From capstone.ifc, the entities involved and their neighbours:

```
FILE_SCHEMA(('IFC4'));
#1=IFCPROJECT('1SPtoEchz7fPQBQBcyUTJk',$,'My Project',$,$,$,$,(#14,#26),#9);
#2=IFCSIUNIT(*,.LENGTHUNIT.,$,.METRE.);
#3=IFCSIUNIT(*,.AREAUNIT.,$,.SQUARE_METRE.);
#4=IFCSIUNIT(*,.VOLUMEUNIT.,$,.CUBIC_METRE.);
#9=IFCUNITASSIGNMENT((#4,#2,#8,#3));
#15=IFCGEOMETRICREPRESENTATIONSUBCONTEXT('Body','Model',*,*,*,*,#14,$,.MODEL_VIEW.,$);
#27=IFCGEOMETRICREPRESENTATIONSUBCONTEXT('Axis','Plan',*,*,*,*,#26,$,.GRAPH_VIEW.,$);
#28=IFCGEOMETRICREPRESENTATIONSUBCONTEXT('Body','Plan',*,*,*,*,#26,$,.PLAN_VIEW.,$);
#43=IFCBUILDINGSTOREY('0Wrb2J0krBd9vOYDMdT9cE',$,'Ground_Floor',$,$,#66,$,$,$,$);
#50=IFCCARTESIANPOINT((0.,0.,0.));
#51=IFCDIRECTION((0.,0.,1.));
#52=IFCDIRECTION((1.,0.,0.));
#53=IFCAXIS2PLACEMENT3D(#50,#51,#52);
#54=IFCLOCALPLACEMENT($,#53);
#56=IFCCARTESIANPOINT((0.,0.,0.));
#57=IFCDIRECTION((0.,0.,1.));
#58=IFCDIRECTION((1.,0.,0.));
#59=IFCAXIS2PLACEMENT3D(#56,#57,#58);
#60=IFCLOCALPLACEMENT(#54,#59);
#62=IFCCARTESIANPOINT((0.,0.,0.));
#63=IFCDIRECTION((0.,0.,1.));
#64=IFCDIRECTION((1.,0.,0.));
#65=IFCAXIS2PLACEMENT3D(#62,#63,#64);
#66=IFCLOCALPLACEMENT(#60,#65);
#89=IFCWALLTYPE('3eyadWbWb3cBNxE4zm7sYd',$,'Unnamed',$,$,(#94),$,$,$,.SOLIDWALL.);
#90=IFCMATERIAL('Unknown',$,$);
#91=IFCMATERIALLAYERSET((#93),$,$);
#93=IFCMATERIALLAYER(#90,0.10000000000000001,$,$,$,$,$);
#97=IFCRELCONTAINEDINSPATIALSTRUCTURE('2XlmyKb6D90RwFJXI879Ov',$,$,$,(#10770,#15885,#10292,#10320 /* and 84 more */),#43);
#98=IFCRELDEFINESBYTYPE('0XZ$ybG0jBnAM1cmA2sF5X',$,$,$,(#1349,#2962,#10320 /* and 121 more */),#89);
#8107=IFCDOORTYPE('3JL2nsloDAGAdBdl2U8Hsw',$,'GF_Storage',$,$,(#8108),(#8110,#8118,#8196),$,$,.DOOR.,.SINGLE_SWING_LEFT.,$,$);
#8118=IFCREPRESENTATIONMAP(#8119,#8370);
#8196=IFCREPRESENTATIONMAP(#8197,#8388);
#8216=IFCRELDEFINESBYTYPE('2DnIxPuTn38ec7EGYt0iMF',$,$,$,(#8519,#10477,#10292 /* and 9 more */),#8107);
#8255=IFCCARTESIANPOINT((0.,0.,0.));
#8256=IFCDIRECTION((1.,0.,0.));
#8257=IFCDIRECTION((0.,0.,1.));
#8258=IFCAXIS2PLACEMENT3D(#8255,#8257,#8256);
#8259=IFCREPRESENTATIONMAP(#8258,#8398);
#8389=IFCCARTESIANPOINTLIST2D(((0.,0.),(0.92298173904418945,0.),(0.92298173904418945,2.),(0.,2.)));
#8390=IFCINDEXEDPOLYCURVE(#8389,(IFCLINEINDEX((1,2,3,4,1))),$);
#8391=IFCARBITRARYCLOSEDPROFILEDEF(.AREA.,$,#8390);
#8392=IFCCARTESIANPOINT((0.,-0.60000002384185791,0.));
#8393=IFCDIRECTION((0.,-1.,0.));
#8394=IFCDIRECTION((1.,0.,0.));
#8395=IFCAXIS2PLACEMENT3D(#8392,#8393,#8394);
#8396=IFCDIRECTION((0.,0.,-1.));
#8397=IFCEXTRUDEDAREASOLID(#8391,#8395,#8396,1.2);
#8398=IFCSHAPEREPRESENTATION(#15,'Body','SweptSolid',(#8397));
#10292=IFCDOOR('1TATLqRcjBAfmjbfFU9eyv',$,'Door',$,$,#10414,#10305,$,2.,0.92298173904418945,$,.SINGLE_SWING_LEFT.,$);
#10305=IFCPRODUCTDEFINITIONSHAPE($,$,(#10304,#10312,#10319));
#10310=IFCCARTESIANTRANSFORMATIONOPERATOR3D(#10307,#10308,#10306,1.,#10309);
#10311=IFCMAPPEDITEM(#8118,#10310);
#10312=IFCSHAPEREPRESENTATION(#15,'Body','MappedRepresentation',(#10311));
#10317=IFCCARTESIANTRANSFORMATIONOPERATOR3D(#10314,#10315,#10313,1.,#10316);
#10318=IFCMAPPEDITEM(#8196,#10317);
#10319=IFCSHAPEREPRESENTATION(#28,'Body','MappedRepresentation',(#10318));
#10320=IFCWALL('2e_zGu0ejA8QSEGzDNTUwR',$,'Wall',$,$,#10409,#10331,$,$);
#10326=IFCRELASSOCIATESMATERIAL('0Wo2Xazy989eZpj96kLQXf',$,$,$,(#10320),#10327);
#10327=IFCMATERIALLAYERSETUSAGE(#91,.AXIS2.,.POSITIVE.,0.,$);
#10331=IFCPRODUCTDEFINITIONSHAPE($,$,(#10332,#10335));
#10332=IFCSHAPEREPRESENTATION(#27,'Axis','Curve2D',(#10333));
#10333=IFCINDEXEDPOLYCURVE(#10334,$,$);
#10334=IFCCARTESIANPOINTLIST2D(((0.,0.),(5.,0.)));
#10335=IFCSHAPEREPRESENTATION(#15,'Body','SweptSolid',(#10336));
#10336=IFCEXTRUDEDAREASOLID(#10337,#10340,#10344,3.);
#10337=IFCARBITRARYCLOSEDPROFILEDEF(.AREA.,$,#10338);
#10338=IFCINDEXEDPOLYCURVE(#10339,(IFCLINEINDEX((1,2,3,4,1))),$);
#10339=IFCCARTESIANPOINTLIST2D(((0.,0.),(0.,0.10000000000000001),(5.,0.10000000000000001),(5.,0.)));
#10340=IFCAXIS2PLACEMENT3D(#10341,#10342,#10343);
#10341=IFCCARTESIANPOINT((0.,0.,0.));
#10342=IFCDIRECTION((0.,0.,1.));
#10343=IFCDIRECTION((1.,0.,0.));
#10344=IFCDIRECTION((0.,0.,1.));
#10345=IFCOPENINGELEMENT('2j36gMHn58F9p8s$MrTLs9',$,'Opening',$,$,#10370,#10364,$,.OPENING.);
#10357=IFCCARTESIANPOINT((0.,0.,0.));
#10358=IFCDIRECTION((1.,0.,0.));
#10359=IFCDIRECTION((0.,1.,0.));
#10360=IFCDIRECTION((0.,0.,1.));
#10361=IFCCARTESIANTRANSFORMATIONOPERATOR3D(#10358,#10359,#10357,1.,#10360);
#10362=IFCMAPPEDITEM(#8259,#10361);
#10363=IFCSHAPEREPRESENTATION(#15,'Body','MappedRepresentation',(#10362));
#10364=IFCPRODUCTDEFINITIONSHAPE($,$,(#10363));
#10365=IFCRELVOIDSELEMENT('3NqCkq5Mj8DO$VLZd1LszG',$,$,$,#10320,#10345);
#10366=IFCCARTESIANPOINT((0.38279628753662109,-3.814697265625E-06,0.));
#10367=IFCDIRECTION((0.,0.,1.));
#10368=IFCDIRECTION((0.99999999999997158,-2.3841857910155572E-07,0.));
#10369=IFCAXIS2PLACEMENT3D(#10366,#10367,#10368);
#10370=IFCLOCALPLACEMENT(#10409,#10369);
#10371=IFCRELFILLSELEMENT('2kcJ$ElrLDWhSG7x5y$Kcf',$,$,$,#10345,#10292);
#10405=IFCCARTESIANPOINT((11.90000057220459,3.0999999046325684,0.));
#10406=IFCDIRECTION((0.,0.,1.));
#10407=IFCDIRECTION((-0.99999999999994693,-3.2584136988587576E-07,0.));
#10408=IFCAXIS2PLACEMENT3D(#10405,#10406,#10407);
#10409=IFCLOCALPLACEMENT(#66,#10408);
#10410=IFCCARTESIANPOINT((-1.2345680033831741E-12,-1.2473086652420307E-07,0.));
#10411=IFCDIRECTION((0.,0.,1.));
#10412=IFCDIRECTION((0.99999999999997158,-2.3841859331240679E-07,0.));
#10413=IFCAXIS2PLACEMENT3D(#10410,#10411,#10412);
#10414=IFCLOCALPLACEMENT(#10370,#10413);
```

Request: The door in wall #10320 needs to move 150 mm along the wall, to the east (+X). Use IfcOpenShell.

```python
import ifcopenshell
import ifcopenshell.api.geometry
import ifcopenshell.util.placement

model = ifcopenshell.open("capstone.ifc")

door = model.by_id(10292)
opening = door.FillsVoids[0].RelatingOpeningElement
wall = opening.VoidsElements[0].RelatingBuildingElement

wall_matrix = ifcopenshell.util.placement.get_local_placement(wall.ObjectPlacement)
shift = wall_matrix[:3, 0] * -0.15
before = ifcopenshell.util.placement.get_local_placement(door.ObjectPlacement)[:3, 3].copy()

# The door is placed relative to its opening, so it follows when the opening moves.
matrix = ifcopenshell.util.placement.get_local_placement(opening.ObjectPlacement)
matrix[:3, 3] += shift
ifcopenshell.api.geometry.edit_object_placement(
    model, product=opening, matrix=matrix, is_si=False, should_transform_children=True
)

after = ifcopenshell.util.placement.get_local_placement(door.ObjectPlacement)[:3, 3]
print("door moved by", (after - before).round(3) + 0.0)

model.write("capstone_v2.ifc")
```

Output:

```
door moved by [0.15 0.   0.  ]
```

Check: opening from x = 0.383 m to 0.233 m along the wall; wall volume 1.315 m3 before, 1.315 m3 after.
